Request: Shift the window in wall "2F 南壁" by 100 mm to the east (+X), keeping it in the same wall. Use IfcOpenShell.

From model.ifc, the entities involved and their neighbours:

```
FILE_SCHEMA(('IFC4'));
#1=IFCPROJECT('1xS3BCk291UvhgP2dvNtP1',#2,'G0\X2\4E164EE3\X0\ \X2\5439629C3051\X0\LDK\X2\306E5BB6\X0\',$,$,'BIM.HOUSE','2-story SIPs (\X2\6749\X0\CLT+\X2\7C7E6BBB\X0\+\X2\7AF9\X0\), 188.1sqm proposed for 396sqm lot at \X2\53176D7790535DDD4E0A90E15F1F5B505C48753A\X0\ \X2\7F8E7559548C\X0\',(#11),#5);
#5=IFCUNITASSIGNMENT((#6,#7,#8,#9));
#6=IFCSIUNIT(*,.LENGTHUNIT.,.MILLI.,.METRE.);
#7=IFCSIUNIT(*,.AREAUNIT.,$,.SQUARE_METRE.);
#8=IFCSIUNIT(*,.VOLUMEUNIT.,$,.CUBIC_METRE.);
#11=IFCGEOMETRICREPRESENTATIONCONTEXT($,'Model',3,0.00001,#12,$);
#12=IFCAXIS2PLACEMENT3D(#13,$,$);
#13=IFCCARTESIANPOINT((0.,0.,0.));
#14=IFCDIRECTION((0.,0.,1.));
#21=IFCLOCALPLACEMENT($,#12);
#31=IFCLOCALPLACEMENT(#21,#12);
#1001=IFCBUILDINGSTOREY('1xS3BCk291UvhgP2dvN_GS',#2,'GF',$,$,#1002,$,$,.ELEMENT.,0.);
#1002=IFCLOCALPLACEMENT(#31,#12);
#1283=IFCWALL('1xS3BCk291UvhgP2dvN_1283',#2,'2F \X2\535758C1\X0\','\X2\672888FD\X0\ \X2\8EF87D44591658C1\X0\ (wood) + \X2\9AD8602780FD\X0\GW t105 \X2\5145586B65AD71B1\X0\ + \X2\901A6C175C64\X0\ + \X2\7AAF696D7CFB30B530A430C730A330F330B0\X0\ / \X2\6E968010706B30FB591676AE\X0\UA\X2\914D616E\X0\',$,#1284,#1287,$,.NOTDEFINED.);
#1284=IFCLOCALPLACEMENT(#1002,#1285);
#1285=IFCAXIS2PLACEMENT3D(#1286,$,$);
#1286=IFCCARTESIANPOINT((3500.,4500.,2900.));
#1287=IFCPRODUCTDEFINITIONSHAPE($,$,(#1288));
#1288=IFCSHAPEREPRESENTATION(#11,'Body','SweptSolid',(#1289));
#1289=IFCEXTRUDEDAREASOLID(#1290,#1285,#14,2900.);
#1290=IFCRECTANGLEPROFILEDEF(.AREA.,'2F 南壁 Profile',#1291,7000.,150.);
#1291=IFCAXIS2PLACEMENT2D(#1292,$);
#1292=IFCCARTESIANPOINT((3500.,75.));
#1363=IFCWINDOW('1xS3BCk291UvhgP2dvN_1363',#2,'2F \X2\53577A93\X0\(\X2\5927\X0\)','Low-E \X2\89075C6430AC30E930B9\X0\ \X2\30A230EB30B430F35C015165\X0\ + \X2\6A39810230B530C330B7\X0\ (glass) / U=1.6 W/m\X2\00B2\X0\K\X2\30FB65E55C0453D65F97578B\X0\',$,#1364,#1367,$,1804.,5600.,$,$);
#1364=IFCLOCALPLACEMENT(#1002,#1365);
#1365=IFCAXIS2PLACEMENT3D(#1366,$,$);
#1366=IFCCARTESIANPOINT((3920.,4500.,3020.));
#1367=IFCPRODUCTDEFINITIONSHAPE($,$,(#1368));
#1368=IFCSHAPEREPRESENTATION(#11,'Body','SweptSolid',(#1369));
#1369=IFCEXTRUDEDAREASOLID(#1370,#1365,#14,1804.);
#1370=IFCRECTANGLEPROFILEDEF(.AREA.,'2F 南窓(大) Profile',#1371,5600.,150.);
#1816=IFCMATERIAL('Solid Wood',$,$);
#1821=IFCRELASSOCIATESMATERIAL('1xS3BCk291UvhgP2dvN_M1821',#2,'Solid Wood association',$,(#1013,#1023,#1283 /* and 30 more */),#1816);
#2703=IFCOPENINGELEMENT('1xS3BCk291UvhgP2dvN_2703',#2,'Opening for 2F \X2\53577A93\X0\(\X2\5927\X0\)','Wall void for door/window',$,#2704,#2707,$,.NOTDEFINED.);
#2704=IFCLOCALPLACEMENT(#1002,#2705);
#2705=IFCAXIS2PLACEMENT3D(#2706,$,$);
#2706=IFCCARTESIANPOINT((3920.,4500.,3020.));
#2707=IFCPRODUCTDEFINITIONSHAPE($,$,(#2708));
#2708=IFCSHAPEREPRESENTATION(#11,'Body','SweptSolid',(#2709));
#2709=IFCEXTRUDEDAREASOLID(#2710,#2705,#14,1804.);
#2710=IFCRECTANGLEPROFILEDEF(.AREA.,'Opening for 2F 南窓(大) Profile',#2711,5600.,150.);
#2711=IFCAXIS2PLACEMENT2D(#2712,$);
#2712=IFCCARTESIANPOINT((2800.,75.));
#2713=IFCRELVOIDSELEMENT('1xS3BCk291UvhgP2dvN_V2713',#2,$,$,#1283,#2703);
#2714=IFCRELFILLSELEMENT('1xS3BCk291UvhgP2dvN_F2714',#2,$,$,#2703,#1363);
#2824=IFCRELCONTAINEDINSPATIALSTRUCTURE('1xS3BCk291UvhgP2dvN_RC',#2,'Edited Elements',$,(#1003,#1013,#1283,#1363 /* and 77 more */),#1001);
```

```python
import ifcopenshell
import ifcopenshell.api.geometry
import ifcopenshell.util.placement
import ifcopenshell.util.unit

model = ifcopenshell.open("model.ifc")
unit_scale = ifcopenshell.util.unit.calculate_unit_scale(model)

window = model.by_guid("1xS3BCk291UvhgP2dvN_1363")
opening = window.FillsVoids[0].RelatingOpeningElement
wall = opening.VoidsElements[0].RelatingBuildingElement

wall_matrix = ifcopenshell.util.placement.get_local_placement(wall.ObjectPlacement)
shift = wall_matrix[:3, 0] * 0.1 / unit_scale
before = ifcopenshell.util.placement.get_local_placement(window.ObjectPlacement)[:3, 3].copy()

# The window is not placed relative to its opening, so move both.
for product in (opening, window):
    matrix = ifcopenshell.util.placement.get_local_placement(product.ObjectPlacement)
    matrix[:3, 3] += shift
    ifcopenshell.api.geometry.edit_object_placement(model, product=product, matrix=matrix, is_si=False)

after = ifcopenshell.util.placement.get_local_placement(window.ObjectPlacement)[:3, 3]
print("window moved by", (after - before).round(3) + 0.0)

model.write("model_updated.ifc")
```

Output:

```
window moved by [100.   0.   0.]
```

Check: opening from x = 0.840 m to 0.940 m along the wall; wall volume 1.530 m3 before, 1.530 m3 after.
